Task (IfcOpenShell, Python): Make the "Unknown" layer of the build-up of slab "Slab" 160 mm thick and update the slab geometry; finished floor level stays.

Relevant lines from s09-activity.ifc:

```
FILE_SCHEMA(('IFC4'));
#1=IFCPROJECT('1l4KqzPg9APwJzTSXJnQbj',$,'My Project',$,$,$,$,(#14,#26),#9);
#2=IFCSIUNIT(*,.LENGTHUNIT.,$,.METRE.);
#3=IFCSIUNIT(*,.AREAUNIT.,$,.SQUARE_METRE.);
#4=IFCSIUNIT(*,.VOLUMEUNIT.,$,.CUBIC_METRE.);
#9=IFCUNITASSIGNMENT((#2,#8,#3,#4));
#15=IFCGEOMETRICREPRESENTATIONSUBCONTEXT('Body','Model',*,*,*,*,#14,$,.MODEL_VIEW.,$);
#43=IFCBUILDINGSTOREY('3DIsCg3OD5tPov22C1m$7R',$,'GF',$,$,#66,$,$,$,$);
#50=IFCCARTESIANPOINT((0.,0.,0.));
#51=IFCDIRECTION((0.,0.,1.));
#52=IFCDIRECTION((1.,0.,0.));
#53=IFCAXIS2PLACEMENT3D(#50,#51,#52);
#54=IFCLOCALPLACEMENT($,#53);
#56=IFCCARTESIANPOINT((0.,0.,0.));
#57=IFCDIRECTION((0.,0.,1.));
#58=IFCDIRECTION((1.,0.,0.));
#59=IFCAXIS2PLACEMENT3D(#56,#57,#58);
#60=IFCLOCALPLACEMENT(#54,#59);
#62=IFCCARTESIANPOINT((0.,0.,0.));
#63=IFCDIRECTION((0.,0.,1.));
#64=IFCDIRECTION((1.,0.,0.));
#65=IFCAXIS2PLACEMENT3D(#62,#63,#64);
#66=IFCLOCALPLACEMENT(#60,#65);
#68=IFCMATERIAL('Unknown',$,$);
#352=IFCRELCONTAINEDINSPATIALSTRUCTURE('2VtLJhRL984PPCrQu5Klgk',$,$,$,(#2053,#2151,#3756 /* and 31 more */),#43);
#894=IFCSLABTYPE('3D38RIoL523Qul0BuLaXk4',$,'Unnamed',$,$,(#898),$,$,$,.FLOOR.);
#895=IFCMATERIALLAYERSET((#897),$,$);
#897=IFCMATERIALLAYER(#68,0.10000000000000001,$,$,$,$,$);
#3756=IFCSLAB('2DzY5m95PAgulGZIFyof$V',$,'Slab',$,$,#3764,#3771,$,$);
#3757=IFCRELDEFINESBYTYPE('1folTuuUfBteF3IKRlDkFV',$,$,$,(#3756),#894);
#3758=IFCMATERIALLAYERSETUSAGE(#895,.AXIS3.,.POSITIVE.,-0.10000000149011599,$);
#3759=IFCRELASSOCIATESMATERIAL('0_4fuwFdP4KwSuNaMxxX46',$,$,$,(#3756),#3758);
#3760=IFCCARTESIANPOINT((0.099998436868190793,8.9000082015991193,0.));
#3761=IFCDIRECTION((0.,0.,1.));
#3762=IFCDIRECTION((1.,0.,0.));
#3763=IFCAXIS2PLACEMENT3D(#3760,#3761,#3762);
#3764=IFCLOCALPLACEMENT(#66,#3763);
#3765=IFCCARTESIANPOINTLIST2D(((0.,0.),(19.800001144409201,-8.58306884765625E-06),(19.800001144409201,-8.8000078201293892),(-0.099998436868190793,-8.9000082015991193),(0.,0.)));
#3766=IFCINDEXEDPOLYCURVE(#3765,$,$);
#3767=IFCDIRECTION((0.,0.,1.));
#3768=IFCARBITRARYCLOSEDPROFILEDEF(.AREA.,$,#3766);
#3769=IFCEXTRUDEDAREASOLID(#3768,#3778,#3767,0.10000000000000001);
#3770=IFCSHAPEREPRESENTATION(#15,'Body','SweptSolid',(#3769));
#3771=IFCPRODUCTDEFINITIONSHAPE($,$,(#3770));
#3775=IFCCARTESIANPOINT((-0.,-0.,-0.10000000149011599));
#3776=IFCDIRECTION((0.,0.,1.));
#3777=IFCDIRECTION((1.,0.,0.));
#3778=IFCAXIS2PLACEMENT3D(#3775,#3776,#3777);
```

```python
import ifcopenshell
import ifcopenshell.util.element
import ifcopenshell.util.representation
import ifcopenshell.util.unit

model = ifcopenshell.open("s09-activity.ifc")
unit_scale = ifcopenshell.util.unit.calculate_unit_scale(model)

layer_set = model.by_id(895)
layer = next(l for l in layer_set.MaterialLayers if l.Material and l.Material.Name == "Unknown")
change = 0.16 / unit_scale - layer.LayerThickness
layer.LayerThickness += change

# Geometry does not follow the layer set by itself.
slabs = [e for e in ifcopenshell.util.element.get_elements_by_material(model, layer_set) if e.is_a("IfcSlab")]
for slab in sorted(slabs, key=lambda e: e.id()):
    body = ifcopenshell.util.representation.get_representation(slab, "Model", "Body")
    solid = body.Items[0]
    old_depth = solid.Depth
    solid.Depth += change
    # Extruded upwards: lower the start of the extrusion so the top stays.
    x, y, z = solid.Position.Location.Coordinates
    solid.Position.Location = model.createIfcCartesianPoint((x, y, z - change))
    print(slab.id(), f"{old_depth:g} -> {solid.Depth:g}")

# The layers are counted up from the underside, which has moved.
for usage in {ifcopenshell.util.element.get_material(slab) for slab in slabs}:
    usage.OffsetFromReferenceLine -= change

model.write("s09-activity_v2.ifc")
```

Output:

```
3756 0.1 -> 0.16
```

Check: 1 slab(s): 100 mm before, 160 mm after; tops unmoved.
